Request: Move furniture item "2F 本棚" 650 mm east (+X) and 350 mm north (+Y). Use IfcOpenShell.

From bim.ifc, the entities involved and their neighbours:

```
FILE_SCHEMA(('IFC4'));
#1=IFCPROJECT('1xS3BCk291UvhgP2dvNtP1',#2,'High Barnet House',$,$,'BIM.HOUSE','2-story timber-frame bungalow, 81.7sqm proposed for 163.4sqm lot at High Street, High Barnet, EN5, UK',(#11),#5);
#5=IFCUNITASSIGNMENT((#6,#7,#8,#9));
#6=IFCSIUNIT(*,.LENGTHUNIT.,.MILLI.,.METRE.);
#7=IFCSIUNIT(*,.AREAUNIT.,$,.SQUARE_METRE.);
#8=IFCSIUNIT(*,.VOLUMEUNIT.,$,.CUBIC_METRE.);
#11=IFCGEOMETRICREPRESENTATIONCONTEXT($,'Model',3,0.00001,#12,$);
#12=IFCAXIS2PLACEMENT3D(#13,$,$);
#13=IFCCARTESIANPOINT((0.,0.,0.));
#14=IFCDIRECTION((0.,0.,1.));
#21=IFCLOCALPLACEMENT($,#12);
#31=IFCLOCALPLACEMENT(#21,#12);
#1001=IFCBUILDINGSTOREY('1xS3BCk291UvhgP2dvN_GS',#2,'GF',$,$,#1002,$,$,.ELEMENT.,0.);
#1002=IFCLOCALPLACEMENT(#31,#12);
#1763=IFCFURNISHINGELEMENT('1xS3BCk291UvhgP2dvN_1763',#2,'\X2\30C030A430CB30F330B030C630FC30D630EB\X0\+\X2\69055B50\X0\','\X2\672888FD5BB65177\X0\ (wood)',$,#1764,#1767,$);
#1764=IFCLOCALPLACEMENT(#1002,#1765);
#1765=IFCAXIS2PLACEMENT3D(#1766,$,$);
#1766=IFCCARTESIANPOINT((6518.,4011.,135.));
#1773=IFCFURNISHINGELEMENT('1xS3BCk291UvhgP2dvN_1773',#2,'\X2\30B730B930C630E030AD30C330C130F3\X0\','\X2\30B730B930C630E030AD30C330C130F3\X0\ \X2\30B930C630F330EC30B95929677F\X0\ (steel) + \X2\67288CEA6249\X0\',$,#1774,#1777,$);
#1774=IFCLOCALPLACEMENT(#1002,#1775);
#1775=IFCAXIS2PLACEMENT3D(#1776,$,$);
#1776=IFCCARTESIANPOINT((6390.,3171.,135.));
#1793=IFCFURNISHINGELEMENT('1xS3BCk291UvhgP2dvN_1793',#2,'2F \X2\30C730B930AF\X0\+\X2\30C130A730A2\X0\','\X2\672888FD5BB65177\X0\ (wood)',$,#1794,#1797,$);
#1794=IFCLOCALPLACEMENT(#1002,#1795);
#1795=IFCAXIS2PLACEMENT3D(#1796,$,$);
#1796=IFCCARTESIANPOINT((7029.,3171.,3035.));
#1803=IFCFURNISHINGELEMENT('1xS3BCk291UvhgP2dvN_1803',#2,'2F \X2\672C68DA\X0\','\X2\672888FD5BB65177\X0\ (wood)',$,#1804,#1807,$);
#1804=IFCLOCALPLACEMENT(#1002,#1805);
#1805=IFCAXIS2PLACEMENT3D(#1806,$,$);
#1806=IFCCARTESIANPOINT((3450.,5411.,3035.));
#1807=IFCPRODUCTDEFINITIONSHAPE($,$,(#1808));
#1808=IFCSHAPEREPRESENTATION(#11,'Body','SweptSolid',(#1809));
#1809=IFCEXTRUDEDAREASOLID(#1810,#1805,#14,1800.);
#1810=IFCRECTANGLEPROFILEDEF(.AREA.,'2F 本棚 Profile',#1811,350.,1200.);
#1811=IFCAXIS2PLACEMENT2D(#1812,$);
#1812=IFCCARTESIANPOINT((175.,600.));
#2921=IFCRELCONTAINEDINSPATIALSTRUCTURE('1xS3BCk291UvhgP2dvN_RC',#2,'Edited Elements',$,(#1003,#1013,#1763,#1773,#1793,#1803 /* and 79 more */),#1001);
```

```python
import ifcopenshell
import ifcopenshell.api.geometry
import ifcopenshell.util.placement
import ifcopenshell.util.unit

model = ifcopenshell.open("bim.ifc")
unit_scale = ifcopenshell.util.unit.calculate_unit_scale(model)

item = model.by_guid("1xS3BCk291UvhgP2dvN_1803")
matrix = ifcopenshell.util.placement.get_local_placement(item.ObjectPlacement)
matrix[0, 3] += 0.65 / unit_scale
matrix[1, 3] += 0.35 / unit_scale
ifcopenshell.api.geometry.edit_object_placement(model, product=item, matrix=matrix, is_si=False)

print(ifcopenshell.util.placement.get_local_placement(item.ObjectPlacement).round(3) + 0.0)

model.write("bim_edited.ifc")
```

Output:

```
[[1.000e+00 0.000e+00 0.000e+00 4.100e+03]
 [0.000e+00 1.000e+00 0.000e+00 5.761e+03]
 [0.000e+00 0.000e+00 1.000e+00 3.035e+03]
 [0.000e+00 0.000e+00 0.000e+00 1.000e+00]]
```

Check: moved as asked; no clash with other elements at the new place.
